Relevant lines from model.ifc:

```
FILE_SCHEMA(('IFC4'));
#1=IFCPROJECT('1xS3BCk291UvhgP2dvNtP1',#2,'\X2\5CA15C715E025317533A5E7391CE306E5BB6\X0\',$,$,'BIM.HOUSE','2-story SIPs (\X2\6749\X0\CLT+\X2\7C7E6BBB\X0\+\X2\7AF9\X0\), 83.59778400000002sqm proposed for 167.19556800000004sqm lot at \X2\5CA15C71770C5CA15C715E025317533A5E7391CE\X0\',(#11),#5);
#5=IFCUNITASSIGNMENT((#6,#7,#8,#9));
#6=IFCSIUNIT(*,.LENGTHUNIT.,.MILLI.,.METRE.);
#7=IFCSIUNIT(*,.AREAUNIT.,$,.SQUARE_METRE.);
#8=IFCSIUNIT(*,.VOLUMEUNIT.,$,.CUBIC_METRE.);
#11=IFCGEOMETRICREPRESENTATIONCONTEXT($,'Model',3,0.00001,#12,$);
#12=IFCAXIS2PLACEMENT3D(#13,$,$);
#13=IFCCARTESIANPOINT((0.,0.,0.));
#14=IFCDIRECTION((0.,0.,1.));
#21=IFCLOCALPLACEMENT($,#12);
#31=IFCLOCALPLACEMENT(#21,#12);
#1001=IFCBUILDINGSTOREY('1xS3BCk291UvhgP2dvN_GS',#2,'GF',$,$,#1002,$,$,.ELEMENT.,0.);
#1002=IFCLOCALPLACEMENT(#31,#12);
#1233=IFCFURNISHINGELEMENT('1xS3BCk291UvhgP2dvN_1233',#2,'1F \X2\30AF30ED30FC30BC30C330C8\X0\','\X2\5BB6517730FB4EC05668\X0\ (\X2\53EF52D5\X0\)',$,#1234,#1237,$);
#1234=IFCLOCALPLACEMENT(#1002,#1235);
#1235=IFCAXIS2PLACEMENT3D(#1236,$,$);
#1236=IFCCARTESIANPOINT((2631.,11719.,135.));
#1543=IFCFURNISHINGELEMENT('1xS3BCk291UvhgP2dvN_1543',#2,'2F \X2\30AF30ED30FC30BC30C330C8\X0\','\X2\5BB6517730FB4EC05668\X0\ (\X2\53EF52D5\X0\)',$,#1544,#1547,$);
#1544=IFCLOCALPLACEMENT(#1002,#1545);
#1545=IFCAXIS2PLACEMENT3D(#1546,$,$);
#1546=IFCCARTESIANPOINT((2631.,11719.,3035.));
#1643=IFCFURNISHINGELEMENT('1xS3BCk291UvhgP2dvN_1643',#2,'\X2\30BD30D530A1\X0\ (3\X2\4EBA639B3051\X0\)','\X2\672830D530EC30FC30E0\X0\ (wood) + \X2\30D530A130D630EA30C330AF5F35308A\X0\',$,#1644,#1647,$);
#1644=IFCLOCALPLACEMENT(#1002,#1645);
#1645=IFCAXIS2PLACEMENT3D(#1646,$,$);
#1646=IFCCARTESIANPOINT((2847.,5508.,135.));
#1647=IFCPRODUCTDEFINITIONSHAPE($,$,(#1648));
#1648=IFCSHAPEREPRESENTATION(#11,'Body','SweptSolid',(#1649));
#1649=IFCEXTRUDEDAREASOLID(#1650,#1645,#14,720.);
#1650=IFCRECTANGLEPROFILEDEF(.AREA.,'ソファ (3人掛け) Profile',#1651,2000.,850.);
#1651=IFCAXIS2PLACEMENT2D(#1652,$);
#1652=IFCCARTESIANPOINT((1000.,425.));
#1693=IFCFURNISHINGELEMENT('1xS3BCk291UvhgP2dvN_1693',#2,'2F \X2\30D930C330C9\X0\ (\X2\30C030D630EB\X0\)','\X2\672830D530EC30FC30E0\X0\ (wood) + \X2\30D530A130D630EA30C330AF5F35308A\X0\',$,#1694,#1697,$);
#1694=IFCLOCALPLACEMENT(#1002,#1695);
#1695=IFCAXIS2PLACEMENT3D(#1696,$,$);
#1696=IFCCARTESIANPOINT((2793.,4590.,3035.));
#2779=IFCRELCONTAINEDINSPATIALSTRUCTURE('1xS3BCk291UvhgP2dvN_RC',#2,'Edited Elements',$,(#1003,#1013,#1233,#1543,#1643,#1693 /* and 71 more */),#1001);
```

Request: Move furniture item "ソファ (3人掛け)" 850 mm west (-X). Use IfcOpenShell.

```python
import ifcopenshell
import ifcopenshell.api.geometry
import ifcopenshell.util.placement
import ifcopenshell.util.unit

model = ifcopenshell.open("model.ifc")
unit_scale = ifcopenshell.util.unit.calculate_unit_scale(model)

item = model.by_guid("1xS3BCk291UvhgP2dvN_1643")
matrix = ifcopenshell.util.placement.get_local_placement(item.ObjectPlacement)
matrix[0, 3] -= 0.85 / unit_scale
ifcopenshell.api.geometry.edit_object_placement(model, product=item, matrix=matrix, is_si=False)

print(ifcopenshell.util.placement.get_local_placement(item.ObjectPlacement).round(3) + 0.0)

model.write("model-out.ifc")
```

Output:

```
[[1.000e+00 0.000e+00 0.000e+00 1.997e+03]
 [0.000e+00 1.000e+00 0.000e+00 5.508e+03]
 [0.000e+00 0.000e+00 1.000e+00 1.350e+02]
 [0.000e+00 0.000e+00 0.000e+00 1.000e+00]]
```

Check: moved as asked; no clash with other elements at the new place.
